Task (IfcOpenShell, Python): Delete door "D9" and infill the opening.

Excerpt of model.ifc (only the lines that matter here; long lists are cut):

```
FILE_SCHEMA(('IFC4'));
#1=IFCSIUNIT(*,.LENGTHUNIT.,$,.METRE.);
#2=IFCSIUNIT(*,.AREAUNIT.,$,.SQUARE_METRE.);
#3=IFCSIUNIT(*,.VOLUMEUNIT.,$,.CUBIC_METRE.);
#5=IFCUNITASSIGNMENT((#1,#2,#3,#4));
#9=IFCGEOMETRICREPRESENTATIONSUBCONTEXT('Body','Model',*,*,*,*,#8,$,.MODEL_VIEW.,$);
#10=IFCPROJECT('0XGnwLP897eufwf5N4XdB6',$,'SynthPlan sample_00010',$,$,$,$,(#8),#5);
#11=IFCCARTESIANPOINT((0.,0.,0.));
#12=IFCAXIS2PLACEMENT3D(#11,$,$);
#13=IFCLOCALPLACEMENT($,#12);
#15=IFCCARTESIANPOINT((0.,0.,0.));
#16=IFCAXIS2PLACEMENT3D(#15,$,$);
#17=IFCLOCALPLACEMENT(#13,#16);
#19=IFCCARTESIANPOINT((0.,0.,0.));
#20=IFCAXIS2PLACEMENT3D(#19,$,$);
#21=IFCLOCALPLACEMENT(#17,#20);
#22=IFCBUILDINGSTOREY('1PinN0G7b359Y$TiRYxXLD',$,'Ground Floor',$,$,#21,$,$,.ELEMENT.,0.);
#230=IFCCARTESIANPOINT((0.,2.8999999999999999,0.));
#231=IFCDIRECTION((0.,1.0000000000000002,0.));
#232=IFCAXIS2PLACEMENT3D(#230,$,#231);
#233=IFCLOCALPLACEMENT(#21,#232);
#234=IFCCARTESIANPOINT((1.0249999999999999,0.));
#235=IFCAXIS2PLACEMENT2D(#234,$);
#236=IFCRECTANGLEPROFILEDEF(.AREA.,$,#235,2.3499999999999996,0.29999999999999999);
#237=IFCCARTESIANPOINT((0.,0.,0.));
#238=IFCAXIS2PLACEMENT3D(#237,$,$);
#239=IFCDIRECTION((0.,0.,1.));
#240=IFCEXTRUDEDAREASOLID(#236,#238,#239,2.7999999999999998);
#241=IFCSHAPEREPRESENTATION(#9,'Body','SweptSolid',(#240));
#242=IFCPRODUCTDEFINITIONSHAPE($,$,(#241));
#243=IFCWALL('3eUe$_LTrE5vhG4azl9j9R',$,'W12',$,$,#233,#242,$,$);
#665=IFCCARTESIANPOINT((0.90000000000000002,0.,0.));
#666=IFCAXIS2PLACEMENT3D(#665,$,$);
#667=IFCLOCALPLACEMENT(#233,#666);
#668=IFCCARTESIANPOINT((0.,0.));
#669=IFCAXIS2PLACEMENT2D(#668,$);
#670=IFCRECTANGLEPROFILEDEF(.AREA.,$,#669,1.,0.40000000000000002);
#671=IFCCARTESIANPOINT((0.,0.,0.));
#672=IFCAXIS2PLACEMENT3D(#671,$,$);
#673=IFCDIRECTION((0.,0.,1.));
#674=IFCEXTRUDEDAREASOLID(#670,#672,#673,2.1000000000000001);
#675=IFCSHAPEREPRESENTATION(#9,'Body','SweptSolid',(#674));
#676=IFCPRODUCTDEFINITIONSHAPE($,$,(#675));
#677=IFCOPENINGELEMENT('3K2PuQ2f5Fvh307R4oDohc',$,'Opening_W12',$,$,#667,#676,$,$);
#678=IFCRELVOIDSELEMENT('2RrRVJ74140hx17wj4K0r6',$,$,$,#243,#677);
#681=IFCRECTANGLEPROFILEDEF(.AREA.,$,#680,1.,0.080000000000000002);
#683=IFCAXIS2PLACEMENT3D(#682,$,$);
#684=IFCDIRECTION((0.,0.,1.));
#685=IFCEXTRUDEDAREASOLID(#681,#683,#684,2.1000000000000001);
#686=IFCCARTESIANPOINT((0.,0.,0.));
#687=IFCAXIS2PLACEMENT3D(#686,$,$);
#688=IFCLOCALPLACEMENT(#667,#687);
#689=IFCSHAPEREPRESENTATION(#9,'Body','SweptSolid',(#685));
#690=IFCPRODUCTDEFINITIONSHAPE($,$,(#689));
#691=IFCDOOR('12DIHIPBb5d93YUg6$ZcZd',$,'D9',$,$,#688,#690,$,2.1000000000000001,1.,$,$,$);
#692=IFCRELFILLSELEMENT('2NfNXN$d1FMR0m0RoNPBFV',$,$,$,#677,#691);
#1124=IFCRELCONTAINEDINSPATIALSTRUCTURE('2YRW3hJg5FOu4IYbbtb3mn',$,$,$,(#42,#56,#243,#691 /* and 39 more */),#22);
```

```python
import ifcopenshell
import ifcopenshell.api.feature
import ifcopenshell.api.root
import ifcopenshell.geom
import ifcopenshell.util.shape

model = ifcopenshell.open("model.ifc")
settings = ifcopenshell.geom.settings()


def volume(element):
    """Net volume in cubic metres, openings subtracted."""
    shape = ifcopenshell.geom.create_shape(settings, element)
    return ifcopenshell.util.shape.get_volume(shape.geometry)


door = model.by_guid("12DIHIPBb5d93YUg6$ZcZd")
opening = door.FillsVoids[0].RelatingOpeningElement
wall = opening.VoidsElements[0].RelatingBuildingElement
before = volume(wall)

ifcopenshell.api.root.remove_product(model, product=door)
ifcopenshell.api.feature.remove_feature(model, feature=opening)

after = volume(wall)

print(f"wall volume {before:.3f} -> {after:.3f} m3")

model.write("model_updated.ifc")
```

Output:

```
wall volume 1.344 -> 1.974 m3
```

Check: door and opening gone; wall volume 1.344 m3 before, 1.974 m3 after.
